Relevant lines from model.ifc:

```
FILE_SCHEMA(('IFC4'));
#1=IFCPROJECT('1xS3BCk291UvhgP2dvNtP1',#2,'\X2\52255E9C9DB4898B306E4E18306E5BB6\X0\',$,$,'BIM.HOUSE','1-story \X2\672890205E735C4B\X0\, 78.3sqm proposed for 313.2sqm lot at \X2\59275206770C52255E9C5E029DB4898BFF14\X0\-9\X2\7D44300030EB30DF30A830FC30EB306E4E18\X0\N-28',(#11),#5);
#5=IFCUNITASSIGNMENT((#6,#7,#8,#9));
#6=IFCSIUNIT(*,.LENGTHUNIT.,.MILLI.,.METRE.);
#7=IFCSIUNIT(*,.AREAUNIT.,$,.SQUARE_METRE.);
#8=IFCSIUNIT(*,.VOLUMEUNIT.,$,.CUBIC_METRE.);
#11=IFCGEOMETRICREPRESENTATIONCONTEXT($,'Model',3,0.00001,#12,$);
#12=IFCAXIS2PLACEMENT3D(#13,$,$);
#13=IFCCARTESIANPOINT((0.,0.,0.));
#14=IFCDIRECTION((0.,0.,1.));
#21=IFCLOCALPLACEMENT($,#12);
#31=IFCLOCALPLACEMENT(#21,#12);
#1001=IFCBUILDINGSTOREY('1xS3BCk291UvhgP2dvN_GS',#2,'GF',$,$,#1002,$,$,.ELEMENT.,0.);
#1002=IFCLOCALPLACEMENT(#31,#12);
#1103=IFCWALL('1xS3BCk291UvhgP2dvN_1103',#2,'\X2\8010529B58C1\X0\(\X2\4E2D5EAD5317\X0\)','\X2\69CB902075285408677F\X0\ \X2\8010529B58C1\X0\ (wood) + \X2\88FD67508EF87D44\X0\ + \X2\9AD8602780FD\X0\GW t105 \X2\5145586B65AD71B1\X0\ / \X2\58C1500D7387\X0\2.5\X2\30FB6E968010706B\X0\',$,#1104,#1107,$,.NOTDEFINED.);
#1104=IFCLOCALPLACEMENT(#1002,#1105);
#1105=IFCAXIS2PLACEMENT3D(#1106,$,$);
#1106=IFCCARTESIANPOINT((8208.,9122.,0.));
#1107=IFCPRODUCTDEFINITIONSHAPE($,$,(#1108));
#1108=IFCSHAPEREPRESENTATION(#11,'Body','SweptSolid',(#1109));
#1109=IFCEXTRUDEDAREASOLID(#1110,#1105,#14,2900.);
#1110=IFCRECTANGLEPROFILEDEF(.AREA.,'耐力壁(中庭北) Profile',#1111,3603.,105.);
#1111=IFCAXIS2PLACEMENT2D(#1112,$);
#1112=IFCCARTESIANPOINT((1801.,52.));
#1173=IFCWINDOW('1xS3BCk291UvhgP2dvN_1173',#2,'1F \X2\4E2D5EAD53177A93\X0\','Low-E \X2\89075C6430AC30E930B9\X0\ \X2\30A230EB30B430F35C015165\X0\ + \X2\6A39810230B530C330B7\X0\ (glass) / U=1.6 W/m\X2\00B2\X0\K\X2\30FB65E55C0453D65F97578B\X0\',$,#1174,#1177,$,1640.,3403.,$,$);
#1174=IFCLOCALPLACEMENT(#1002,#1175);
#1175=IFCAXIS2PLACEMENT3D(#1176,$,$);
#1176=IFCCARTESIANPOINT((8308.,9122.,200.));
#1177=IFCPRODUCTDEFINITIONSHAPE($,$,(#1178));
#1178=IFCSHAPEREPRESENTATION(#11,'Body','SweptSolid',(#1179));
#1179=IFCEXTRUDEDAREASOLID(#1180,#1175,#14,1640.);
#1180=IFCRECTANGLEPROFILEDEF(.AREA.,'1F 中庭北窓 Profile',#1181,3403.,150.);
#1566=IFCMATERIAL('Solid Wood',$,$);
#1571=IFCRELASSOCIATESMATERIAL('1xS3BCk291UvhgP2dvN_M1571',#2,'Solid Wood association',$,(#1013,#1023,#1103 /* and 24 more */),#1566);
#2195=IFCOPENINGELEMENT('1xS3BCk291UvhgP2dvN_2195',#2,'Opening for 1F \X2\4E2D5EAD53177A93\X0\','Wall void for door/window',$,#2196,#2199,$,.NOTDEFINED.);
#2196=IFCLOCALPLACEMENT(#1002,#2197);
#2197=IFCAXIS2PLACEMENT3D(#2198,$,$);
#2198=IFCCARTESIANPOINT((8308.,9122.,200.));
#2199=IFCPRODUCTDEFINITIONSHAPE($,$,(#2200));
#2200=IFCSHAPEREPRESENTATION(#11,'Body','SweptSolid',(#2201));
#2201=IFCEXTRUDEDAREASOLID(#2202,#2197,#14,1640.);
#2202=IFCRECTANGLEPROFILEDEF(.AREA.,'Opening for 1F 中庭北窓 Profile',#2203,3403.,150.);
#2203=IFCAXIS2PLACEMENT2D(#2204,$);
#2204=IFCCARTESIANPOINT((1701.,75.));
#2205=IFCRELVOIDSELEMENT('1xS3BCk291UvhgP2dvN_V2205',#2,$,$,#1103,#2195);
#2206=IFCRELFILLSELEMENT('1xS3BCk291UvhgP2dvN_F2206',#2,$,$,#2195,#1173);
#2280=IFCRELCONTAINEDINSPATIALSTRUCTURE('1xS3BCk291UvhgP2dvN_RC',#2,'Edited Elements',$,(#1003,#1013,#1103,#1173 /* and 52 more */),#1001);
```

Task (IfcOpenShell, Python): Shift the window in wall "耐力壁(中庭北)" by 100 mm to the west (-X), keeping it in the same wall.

```python
import ifcopenshell
import ifcopenshell.api.geometry
import ifcopenshell.util.placement
import ifcopenshell.util.unit

model = ifcopenshell.open("model.ifc")
unit_scale = ifcopenshell.util.unit.calculate_unit_scale(model)

window = model.by_guid("1xS3BCk291UvhgP2dvN_1173")
opening = window.FillsVoids[0].RelatingOpeningElement
wall = opening.VoidsElements[0].RelatingBuildingElement

wall_matrix = ifcopenshell.util.placement.get_local_placement(wall.ObjectPlacement)
shift = wall_matrix[:3, 0] * -0.1 / unit_scale
before = ifcopenshell.util.placement.get_local_placement(window.ObjectPlacement)[:3, 3].copy()

# The window is not placed relative to its opening, so move both.
for product in (opening, window):
    matrix = ifcopenshell.util.placement.get_local_placement(product.ObjectPlacement)
    matrix[:3, 3] += shift
    ifcopenshell.api.geometry.edit_object_placement(model, product=product, matrix=matrix, is_si=False)

after = ifcopenshell.util.placement.get_local_placement(window.ObjectPlacement)[:3, 3]
print("window moved by", (after - before).round(3) + 0.0)

model.write("model_updated.ifc")
```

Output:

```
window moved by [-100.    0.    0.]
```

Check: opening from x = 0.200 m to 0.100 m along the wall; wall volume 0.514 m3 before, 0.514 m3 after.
